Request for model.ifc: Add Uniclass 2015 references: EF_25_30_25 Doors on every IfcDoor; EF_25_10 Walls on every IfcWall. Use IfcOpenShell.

First a look at what the model holds.

```python
import ifcopenshell

model = ifcopenshell.open("model.ifc")
print(model.schema)
print("classifications:", [c.Name for c in model.by_type("IfcClassification")])
for ifc_class in ("IfcDoor", "IfcRoof", "IfcStair", "IfcWall", "IfcWindow"):
    print(ifc_class, len(model.by_type(ifc_class)))
```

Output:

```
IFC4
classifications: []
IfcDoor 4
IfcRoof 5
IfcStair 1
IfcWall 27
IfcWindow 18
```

```python
import ifcopenshell
import ifcopenshell.api.classification

model = ifcopenshell.open("model.ifc")

system = ifcopenshell.api.classification.add_classification(model, classification="Uniclass 2015")

codes = {
    "IfcDoor": ("EF_25_30_25", "Doors"),
    "IfcWall": ("EF_25_10", "Walls"),
}
for ifc_class, (code, name) in codes.items():
    products = model.by_type(ifc_class)
    ifcopenshell.api.classification.add_reference(
        model, products=products, classification=system, identification=code, name=name
    )
    print(code, len(products))

model.write("model_edited.ifc")
```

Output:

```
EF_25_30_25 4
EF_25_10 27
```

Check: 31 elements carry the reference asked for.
